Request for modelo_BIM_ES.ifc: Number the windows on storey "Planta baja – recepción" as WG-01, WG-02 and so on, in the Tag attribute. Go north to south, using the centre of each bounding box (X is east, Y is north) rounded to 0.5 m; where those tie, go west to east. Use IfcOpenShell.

First a look at what the model holds.

```python
import ifcopenshell
import ifcopenshell.util.element
import ifcopenshell.util.placement

model = ifcopenshell.open("modelo_BIM_ES.ifc")
print(model.schema)
storey = next(s for s in model.by_type("IfcBuildingStorey") if s.Name == "Planta baja – recepción")
windows = [e for e in ifcopenshell.util.element.get_decomposition(storey) if e.is_a("IfcWindow")]
for e in sorted(windows, key=lambda e: e.id()):
    origin = ifcopenshell.util.placement.get_local_placement(e.ObjectPlacement)[:3, 3]
    print(e.id(), e.Tag, e.Name, origin.round(2) + 0.0, sep=" | ")
```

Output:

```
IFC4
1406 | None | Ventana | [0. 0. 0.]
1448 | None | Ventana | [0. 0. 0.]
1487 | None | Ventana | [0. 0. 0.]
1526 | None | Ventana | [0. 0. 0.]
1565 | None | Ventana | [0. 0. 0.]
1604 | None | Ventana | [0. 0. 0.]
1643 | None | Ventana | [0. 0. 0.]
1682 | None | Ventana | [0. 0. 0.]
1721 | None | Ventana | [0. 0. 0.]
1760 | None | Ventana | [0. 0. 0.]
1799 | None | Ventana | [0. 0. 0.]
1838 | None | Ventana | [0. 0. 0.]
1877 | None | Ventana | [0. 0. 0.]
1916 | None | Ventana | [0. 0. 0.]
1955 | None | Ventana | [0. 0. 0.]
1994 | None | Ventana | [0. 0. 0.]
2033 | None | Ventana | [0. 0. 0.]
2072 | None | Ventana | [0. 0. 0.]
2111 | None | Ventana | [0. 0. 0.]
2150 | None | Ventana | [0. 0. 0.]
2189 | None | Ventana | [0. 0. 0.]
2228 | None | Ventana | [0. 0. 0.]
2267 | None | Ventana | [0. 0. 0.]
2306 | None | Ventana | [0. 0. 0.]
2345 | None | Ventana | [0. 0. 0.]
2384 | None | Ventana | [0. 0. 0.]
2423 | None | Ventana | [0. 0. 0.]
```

```python
import ifcopenshell
import ifcopenshell.geom
import ifcopenshell.util.element
import ifcopenshell.util.shape

model = ifcopenshell.open("modelo_BIM_ES.ifc")
settings = ifcopenshell.geom.settings()
settings.set("use-world-coords", True)


def centre(element):
    shape = ifcopenshell.geom.create_shape(settings, element)
    return ifcopenshell.util.shape.get_bbox_centroid(shape.geometry)


storey = next(s for s in model.by_type("IfcBuildingStorey") if s.Name == "Planta baja – recepción")
windows = [e for e in ifcopenshell.util.element.get_decomposition(storey) if e.is_a("IfcWindow")]

# Insertion points can sit at a corner or the storey origin, so sort by the geometry (in metres).
centres = {e: centre(e) for e in windows}
windows.sort(key=lambda e: (-round(centres[e][1] / 0.5), centres[e][0]))

for i, e in enumerate(windows, start=1):
    number = f"WG-{i:02d}"
    e.Tag = number
    print(e.id(), number)

model.write("modelo_BIM_ES-out.ifc")
```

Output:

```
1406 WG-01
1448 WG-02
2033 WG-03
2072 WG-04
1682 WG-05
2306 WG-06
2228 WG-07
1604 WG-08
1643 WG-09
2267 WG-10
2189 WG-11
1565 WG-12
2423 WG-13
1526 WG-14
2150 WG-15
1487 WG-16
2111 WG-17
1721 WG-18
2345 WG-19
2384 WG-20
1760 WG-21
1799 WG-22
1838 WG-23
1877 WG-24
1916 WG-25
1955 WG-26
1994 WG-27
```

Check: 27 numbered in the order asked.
